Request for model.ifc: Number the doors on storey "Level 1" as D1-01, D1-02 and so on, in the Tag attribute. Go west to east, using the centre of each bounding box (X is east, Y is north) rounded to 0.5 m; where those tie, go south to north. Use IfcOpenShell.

First a look at what the model holds.

```python
import ifcopenshell
import ifcopenshell.util.element
import ifcopenshell.util.placement

model = ifcopenshell.open("model.ifc")
print(model.schema)
storey = next(s for s in model.by_type("IfcBuildingStorey") if s.Name == "Level 1")
doors = [e for e in ifcopenshell.util.element.get_decomposition(storey) if e.is_a("IfcDoor")]
for e in sorted(doors, key=lambda e: e.id()):
    origin = ifcopenshell.util.placement.get_local_placement(e.ObjectPlacement)[:3, 3]
    print(e.id(), e.Tag, e.Name, origin.round(2) + 0.0, sep=" | ")
```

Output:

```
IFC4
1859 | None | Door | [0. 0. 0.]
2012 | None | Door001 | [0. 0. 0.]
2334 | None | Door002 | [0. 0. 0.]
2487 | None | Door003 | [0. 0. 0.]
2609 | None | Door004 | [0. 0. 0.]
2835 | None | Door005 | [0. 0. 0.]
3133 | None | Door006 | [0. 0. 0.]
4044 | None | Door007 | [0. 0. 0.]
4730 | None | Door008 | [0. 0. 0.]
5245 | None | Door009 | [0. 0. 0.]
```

```python
import ifcopenshell
import ifcopenshell.geom
import ifcopenshell.util.element
import ifcopenshell.util.shape

model = ifcopenshell.open("model.ifc")
settings = ifcopenshell.geom.settings()
settings.set("use-world-coords", True)


def centre(element):
    shape = ifcopenshell.geom.create_shape(settings, element)
    return ifcopenshell.util.shape.get_bbox_centroid(shape.geometry)


storey = next(s for s in model.by_type("IfcBuildingStorey") if s.Name == "Level 1")
doors = [e for e in ifcopenshell.util.element.get_decomposition(storey) if e.is_a("IfcDoor")]

# Insertion points can sit at a corner or the storey origin, so sort by the geometry (in metres).
centres = {e: centre(e) for e in doors}
doors.sort(key=lambda e: (round(centres[e][0] / 0.5), centres[e][1]))

for i, e in enumerate(doors, start=1):
    number = f"D1-{i:02d}"
    e.Tag = number
    print(e.id(), number)

model.write("model-out.ifc")
```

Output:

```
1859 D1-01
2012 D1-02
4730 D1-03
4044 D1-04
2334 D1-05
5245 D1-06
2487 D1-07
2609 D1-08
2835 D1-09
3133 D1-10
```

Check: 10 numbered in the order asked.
